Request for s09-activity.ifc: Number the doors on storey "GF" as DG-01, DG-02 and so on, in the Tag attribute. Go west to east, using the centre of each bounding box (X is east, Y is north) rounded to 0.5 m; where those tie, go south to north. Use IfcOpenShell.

First a look at what the model holds.

```python
import ifcopenshell
import ifcopenshell.util.element
import ifcopenshell.util.placement

model = ifcopenshell.open("s09-activity.ifc")
print(model.schema)
storey = next(s for s in model.by_type("IfcBuildingStorey") if s.Name == "GF")
doors = [e for e in ifcopenshell.util.element.get_decomposition(storey) if e.is_a("IfcDoor")]
for e in sorted(doors, key=lambda e: e.id()):
    origin = ifcopenshell.util.placement.get_local_placement(e.ObjectPlacement)[:3, 3]
    print(e.id(), e.Tag, e.Name, origin.round(2) + 0.0, sep=" | ")
```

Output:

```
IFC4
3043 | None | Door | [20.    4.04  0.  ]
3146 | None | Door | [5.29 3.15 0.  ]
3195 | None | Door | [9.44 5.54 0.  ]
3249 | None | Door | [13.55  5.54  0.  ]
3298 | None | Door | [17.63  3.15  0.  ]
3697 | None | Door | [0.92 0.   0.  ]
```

```python
import ifcopenshell
import ifcopenshell.geom
import ifcopenshell.util.element
import ifcopenshell.util.shape

model = ifcopenshell.open("s09-activity.ifc")
settings = ifcopenshell.geom.settings()
settings.set("use-world-coords", True)


def centre(element):
    shape = ifcopenshell.geom.create_shape(settings, element)
    return ifcopenshell.util.shape.get_bbox_centroid(shape.geometry)


storey = next(s for s in model.by_type("IfcBuildingStorey") if s.Name == "GF")
doors = [e for e in ifcopenshell.util.element.get_decomposition(storey) if e.is_a("IfcDoor")]

# Insertion points can sit at a corner or the storey origin, so sort by the geometry (in metres).
centres = {e: centre(e) for e in doors}
doors.sort(key=lambda e: (round(centres[e][0] / 0.5), centres[e][1]))

for i, e in enumerate(doors, start=1):
    number = f"DG-{i:02d}"
    e.Tag = number
    print(e.id(), number)

model.write("s09-activity_v2.ifc")
```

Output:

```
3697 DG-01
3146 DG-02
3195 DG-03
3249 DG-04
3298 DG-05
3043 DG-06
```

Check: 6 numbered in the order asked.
